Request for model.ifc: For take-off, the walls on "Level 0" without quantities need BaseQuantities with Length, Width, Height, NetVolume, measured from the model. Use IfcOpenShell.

First a look at what the model holds.

```python
import ifcopenshell
import ifcopenshell.util.element
import ifcopenshell.util.unit

model = ifcopenshell.open("model.ifc")
print(model.schema)
for unit_type in ("LENGTHUNIT", "AREAUNIT", "VOLUMEUNIT"):
    print(unit_type, ifcopenshell.util.unit.calculate_unit_scale(model, unit_type))
storey = next(s for s in model.by_type("IfcBuildingStorey") if s.Name == "Level 0")
walls = [e for e in ifcopenshell.util.element.get_decomposition(storey) if e.is_a("IfcWall")]
for e in sorted(walls, key=lambda e: e.id()):
    print(e.id(), e.is_a(), e.Name, list(ifcopenshell.util.element.get_psets(e, qtos_only=True)), sep=" | ")
```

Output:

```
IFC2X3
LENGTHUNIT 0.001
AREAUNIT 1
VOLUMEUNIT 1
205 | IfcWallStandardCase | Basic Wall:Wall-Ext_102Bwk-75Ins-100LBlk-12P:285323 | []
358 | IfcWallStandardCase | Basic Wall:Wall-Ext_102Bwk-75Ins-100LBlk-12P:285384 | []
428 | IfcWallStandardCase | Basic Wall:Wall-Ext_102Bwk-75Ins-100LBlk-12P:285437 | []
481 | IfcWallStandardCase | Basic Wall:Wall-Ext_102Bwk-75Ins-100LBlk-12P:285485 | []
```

```python
import ifcopenshell
import ifcopenshell.api.pset
import ifcopenshell.geom
import ifcopenshell.util.element
import ifcopenshell.util.shape
import ifcopenshell.util.unit

model = ifcopenshell.open("model.ifc")
unit_scale = ifcopenshell.util.unit.calculate_unit_scale(model)
volume_scale = ifcopenshell.util.unit.calculate_unit_scale(model, "VOLUMEUNIT")
settings = ifcopenshell.geom.settings()

storey = next(s for s in model.by_type("IfcBuildingStorey") if s.Name == "Level 0")
walls = [e for e in ifcopenshell.util.element.get_decomposition(storey) if e.is_a("IfcWall")]

for e in sorted(walls, key=lambda e: e.id()):
    if ifcopenshell.util.element.get_psets(e, qtos_only=True, should_inherit=False):
        continue
    # Geometry comes back in metres, in the element's own axes.
    shape = ifcopenshell.geom.create_shape(settings, e)
    values = {
        "Length": ifcopenshell.util.shape.get_x(shape.geometry) / unit_scale,
        "Width": ifcopenshell.util.shape.get_y(shape.geometry) / unit_scale,
        "Height": ifcopenshell.util.shape.get_z(shape.geometry) / unit_scale,
        "NetVolume": ifcopenshell.util.shape.get_volume(shape.geometry) / volume_scale,
    }
    qto = ifcopenshell.api.pset.add_qto(model, product=e, name="BaseQuantities")
    ifcopenshell.api.pset.edit_qto(model, qto=qto, properties=values)
    print(e.id(), {k: round(v, 3) for k, v in values.items()})

model.write("model_edited.ifc")
```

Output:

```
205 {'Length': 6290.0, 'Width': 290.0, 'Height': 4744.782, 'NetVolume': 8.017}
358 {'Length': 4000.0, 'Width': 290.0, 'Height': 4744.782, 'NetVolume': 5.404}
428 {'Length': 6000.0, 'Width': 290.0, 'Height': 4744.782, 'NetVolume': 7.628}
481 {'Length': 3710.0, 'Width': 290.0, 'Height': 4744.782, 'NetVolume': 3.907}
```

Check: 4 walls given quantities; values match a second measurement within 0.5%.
